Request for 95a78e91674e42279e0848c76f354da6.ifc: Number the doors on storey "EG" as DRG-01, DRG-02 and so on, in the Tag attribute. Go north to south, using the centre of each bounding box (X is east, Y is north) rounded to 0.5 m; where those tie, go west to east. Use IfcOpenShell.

First a look at what the model holds.

```python
import ifcopenshell
import ifcopenshell.util.element
import ifcopenshell.util.placement

model = ifcopenshell.open("95a78e91674e42279e0848c76f354da6.ifc")
print(model.schema)
storey = next(s for s in model.by_type("IfcBuildingStorey") if s.Name == "EG")
doors = [e for e in ifcopenshell.util.element.get_decomposition(storey) if e.is_a("IfcDoor")]
for e in sorted(doors, key=lambda e: e.id()):
    origin = ifcopenshell.util.placement.get_local_placement(e.ObjectPlacement)[:3, 3]
    print(e.id(), e.Tag, e.Name, origin.round(2) + 0.0, sep=" | ")
```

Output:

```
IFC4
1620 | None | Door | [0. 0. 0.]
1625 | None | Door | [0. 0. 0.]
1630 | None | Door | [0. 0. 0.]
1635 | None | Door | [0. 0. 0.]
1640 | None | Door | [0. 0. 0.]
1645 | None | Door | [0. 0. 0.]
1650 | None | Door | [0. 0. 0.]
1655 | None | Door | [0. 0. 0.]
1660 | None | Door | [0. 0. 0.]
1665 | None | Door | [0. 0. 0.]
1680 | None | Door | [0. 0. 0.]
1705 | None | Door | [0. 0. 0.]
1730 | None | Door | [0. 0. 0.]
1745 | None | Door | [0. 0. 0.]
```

```python
import ifcopenshell
import ifcopenshell.geom
import ifcopenshell.util.element
import ifcopenshell.util.shape

model = ifcopenshell.open("95a78e91674e42279e0848c76f354da6.ifc")
settings = ifcopenshell.geom.settings()
settings.set("use-world-coords", True)


def centre(element):
    shape = ifcopenshell.geom.create_shape(settings, element)
    return ifcopenshell.util.shape.get_bbox_centroid(shape.geometry)


storey = next(s for s in model.by_type("IfcBuildingStorey") if s.Name == "EG")
doors = [e for e in ifcopenshell.util.element.get_decomposition(storey) if e.is_a("IfcDoor")]

# Insertion points can sit at a corner or the storey origin, so sort by the geometry (in metres).
centres = {e: centre(e) for e in doors}
doors.sort(key=lambda e: (-round(centres[e][1] / 0.5), centres[e][0]))

for i, e in enumerate(doors, start=1):
    number = f"DRG-{i:02d}"
    e.Tag = number
    print(e.id(), number)

model.write("95a78e91674e42279e0848c76f354da6-out.ifc")
```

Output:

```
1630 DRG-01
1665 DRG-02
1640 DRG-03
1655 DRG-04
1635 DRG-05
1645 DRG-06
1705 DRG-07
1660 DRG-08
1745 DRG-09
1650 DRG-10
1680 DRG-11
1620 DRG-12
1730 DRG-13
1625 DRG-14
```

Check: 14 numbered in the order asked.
